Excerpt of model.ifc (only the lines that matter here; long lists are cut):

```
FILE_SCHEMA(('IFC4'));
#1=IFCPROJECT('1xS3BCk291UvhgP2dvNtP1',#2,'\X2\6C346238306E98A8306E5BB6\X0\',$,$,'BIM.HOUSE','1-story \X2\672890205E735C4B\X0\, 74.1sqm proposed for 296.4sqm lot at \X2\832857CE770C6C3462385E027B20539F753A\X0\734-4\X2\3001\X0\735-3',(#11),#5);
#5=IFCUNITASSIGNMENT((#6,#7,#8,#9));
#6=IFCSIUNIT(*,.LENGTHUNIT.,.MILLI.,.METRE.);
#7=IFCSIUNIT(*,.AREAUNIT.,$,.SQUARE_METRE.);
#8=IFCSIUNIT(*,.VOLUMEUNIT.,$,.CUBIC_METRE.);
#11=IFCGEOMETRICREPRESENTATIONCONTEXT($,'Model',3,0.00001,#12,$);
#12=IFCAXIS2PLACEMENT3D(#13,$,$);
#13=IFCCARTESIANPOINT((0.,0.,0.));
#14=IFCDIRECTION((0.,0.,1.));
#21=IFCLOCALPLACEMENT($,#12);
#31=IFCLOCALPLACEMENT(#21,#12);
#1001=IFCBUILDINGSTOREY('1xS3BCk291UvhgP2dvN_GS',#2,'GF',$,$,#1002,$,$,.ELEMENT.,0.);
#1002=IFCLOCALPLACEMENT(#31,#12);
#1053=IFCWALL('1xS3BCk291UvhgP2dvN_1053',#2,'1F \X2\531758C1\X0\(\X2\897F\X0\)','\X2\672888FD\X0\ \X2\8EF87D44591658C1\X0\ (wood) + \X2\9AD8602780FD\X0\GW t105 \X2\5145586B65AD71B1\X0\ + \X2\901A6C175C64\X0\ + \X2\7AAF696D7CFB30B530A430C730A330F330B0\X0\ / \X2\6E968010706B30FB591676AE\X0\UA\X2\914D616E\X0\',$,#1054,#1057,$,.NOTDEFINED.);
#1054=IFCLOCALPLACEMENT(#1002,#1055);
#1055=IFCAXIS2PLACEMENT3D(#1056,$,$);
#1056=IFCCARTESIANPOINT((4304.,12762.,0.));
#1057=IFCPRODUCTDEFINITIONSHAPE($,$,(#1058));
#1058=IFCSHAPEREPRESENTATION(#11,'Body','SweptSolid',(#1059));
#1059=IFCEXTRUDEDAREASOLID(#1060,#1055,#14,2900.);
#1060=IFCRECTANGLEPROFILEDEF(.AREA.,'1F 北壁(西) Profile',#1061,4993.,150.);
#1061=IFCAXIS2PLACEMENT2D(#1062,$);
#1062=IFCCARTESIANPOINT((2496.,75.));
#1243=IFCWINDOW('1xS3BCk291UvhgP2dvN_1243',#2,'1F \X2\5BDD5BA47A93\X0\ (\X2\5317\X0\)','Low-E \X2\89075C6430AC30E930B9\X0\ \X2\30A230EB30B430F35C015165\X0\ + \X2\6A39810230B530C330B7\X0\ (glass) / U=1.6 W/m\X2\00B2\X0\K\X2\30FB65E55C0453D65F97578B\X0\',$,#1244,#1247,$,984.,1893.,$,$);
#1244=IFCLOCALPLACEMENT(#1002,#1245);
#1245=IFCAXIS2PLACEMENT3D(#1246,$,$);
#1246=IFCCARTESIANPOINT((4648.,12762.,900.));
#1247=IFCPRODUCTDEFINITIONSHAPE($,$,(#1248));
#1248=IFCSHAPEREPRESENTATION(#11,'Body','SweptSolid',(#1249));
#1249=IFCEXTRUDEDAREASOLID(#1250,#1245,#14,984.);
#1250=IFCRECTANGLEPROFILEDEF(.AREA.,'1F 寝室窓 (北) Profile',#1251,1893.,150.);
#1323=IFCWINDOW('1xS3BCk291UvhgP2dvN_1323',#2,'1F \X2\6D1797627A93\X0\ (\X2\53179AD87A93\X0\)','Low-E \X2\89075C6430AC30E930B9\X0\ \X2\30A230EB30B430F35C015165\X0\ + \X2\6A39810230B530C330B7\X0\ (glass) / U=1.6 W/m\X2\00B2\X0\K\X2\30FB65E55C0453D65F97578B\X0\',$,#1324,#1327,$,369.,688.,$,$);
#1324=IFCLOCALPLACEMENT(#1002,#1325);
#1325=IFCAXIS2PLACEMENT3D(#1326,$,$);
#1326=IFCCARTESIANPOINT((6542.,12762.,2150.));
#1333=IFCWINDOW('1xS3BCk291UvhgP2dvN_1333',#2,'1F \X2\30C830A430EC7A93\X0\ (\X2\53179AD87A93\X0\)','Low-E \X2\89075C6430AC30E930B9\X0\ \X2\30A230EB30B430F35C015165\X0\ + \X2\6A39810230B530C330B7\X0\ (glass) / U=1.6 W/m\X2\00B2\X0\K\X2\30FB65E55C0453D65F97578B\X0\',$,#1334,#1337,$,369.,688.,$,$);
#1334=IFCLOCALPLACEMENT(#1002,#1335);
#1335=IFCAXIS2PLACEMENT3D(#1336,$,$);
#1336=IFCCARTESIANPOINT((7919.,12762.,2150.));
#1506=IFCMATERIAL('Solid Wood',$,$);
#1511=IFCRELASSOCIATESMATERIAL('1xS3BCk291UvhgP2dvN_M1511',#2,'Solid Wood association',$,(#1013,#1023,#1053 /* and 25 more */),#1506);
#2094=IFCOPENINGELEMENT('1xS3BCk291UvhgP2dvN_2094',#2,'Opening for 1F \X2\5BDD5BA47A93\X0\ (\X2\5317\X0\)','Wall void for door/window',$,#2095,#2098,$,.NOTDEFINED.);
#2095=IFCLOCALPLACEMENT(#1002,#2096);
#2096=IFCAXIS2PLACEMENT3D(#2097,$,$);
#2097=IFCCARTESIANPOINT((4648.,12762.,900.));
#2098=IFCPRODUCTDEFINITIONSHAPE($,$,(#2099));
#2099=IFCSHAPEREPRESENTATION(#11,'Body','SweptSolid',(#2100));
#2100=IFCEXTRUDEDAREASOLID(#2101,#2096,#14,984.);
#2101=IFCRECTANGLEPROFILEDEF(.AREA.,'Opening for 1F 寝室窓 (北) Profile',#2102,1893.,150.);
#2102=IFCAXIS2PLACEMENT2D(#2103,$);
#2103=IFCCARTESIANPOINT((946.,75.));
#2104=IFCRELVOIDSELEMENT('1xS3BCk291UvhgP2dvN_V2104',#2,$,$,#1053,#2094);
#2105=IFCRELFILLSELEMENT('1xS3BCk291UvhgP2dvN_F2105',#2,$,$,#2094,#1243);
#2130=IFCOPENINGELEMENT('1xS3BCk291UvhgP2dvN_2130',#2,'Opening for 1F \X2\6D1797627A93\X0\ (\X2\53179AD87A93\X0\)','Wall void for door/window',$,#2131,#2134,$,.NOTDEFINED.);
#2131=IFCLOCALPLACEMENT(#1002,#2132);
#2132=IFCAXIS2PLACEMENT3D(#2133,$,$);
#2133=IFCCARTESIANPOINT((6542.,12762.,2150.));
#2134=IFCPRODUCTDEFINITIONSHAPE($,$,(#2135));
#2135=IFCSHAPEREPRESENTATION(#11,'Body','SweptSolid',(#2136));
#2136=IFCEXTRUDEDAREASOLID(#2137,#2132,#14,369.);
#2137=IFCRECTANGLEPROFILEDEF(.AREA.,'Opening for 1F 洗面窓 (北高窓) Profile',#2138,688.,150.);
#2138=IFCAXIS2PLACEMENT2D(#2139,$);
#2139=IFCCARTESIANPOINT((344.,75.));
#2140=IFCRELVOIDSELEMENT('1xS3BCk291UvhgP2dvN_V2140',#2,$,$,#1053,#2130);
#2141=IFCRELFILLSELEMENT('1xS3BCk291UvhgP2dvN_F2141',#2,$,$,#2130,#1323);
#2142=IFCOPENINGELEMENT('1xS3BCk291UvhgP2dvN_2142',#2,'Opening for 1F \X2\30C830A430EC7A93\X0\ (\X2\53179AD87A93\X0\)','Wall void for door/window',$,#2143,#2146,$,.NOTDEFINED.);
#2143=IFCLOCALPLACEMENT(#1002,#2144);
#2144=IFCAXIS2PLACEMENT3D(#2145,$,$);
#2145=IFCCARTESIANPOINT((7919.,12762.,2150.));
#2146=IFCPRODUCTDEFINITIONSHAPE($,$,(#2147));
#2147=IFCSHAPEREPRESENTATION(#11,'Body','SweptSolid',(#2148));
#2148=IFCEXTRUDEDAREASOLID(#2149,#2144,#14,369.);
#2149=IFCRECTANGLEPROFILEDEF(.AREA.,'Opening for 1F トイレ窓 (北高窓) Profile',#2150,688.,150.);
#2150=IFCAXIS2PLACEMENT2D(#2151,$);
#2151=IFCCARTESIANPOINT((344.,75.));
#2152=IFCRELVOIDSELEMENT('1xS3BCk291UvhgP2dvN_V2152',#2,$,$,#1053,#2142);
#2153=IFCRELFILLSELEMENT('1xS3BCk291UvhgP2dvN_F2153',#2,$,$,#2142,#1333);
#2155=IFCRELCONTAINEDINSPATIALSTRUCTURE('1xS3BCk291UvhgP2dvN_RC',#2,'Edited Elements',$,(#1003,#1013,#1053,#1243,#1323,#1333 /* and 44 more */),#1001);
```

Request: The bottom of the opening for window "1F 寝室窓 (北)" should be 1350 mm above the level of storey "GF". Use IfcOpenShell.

```python
import numpy as np
import ifcopenshell
import ifcopenshell.api.geometry
import ifcopenshell.geom
import ifcopenshell.util.element
import ifcopenshell.util.placement
import ifcopenshell.util.shape
import ifcopenshell.util.unit

model = ifcopenshell.open("model.ifc")
unit_scale = ifcopenshell.util.unit.calculate_unit_scale(model)

window = model.by_guid("1xS3BCk291UvhgP2dvN_1243")
opening = window.FillsVoids[0].RelatingOpeningElement
storey = ifcopenshell.util.element.get_container(window, ifc_class="IfcBuildingStorey")
level = ifcopenshell.util.placement.get_local_placement(storey.ObjectPlacement)[2, 3]

# The opening's origin need not be at the sill, so measure its lowest point.
shape = ifcopenshell.geom.create_shape(ifcopenshell.geom.settings(), opening)
bottom = ifcopenshell.util.shape.get_shape_bottom_elevation(shape, shape.geometry) / unit_scale
dz = level + 1350.0 - bottom

shift = np.array([0.0, 0.0, dz])
# The window is not placed relative to its opening, so move both.
for product in (opening, window):
    matrix = ifcopenshell.util.placement.get_local_placement(product.ObjectPlacement)
    matrix[:3, 3] += shift
    ifcopenshell.api.geometry.edit_object_placement(model, product=product, matrix=matrix, is_si=False)

print(f"moved by {dz * unit_scale:+.3f} m")

model.write("model_updated.ifc")
```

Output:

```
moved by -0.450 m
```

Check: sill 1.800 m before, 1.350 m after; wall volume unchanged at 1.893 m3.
